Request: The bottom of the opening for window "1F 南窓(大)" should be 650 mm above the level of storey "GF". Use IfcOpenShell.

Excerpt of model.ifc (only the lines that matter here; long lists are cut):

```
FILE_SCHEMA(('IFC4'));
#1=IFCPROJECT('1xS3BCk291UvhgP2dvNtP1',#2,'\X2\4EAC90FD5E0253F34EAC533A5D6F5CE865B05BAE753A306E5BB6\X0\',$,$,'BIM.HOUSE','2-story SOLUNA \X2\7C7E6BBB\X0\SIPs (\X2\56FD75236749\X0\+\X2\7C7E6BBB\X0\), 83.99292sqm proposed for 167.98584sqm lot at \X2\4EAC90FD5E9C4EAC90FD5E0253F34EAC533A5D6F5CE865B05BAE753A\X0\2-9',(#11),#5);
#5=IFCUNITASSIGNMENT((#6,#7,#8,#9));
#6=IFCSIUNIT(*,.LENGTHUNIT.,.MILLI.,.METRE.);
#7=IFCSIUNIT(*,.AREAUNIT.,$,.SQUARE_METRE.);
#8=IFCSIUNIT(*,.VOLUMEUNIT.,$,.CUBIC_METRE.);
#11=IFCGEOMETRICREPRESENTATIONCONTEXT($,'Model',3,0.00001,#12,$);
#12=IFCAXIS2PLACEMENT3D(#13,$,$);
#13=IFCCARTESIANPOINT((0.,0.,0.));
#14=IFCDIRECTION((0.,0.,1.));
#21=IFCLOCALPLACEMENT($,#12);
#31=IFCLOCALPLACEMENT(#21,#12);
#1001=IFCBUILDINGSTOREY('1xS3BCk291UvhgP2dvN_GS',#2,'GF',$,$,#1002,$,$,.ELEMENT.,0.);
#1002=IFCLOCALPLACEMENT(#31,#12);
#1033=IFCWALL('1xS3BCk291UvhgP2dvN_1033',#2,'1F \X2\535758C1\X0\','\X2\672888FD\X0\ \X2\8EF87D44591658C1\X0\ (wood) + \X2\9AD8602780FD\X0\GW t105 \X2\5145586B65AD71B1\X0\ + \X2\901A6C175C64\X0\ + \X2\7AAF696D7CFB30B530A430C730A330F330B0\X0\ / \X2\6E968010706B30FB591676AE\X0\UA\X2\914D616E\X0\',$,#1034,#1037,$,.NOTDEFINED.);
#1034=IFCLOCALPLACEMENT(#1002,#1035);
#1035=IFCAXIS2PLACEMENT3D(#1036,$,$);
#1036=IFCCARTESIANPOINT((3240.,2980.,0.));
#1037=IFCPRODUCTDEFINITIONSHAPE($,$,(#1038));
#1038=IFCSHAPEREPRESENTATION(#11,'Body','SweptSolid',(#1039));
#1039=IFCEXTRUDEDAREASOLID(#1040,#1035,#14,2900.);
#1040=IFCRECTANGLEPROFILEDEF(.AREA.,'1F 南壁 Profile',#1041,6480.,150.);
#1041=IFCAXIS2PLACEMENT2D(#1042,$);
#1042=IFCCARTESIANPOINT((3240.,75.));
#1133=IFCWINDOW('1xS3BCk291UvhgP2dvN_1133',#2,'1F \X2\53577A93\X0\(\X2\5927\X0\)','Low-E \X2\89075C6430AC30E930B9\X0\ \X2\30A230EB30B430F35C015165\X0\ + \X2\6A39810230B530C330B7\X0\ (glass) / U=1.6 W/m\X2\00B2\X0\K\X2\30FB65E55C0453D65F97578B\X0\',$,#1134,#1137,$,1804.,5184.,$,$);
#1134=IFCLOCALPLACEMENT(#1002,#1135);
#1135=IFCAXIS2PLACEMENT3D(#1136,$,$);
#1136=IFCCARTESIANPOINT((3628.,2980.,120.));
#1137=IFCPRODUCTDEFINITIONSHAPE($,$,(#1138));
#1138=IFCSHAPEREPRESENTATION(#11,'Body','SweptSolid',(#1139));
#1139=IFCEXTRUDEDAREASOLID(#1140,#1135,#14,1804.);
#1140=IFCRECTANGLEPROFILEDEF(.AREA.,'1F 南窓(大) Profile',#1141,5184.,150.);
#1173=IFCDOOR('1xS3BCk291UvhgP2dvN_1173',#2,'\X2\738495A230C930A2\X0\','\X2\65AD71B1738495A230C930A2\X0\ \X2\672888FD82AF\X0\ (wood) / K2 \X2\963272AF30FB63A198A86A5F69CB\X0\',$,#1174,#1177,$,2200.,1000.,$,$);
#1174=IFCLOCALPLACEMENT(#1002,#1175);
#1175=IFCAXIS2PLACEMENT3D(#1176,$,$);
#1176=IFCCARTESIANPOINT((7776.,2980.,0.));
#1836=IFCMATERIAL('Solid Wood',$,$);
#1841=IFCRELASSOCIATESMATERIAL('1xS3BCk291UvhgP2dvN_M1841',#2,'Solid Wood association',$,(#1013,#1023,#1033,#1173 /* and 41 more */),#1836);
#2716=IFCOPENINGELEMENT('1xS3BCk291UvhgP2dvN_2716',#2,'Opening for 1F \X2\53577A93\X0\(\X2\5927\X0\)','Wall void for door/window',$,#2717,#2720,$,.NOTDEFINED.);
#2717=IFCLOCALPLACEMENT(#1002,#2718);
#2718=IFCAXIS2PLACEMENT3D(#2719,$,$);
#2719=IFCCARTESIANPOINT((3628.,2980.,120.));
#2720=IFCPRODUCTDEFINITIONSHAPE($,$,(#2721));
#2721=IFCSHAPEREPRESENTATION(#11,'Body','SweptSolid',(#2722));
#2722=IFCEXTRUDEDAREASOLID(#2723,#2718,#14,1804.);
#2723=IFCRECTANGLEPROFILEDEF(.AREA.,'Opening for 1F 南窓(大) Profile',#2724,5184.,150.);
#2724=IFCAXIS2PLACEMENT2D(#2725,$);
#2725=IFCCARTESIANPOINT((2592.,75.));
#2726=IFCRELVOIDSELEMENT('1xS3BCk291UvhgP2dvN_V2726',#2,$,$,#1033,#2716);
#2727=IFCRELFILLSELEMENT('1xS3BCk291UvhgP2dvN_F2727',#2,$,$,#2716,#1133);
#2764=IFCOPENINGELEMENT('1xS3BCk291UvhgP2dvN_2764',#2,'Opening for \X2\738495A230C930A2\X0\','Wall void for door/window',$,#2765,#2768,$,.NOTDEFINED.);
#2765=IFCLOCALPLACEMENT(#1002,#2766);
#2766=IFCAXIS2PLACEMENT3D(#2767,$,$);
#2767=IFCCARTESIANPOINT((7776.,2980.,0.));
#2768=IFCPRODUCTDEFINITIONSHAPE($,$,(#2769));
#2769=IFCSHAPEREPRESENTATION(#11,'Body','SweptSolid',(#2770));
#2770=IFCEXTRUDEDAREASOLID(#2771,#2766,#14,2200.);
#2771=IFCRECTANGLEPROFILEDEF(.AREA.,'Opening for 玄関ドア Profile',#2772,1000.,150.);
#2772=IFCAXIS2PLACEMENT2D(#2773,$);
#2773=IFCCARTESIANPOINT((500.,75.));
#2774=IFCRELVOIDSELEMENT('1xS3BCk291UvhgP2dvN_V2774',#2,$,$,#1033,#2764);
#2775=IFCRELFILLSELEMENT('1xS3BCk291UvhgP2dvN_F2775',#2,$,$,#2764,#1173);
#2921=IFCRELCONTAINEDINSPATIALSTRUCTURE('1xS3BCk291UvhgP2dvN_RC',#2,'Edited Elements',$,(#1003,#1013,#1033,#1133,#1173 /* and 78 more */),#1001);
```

```python
import numpy as np
import ifcopenshell
import ifcopenshell.api.geometry
import ifcopenshell.geom
import ifcopenshell.util.element
import ifcopenshell.util.placement
import ifcopenshell.util.shape
import ifcopenshell.util.unit

model = ifcopenshell.open("model.ifc")
unit_scale = ifcopenshell.util.unit.calculate_unit_scale(model)

window = model.by_id(1133)
opening = window.FillsVoids[0].RelatingOpeningElement
storey = ifcopenshell.util.element.get_container(window, ifc_class="IfcBuildingStorey")
level = ifcopenshell.util.placement.get_local_placement(storey.ObjectPlacement)[2, 3]

# The opening's origin need not be at the sill, so measure its lowest point.
shape = ifcopenshell.geom.create_shape(ifcopenshell.geom.settings(), opening)
bottom = ifcopenshell.util.shape.get_shape_bottom_elevation(shape, shape.geometry) / unit_scale
dz = level + 650.0 - bottom

shift = np.array([0.0, 0.0, dz])
# The window is not placed relative to its opening, so move both.
for product in (opening, window):
    matrix = ifcopenshell.util.placement.get_local_placement(product.ObjectPlacement)
    matrix[:3, 3] += shift
    ifcopenshell.api.geometry.edit_object_placement(model, product=product, matrix=matrix, is_si=False)

print(f"moved by {dz * unit_scale:+.3f} m")

model.write("model_updated.ifc")
```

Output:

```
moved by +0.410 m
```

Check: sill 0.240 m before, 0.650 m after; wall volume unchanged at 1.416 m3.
